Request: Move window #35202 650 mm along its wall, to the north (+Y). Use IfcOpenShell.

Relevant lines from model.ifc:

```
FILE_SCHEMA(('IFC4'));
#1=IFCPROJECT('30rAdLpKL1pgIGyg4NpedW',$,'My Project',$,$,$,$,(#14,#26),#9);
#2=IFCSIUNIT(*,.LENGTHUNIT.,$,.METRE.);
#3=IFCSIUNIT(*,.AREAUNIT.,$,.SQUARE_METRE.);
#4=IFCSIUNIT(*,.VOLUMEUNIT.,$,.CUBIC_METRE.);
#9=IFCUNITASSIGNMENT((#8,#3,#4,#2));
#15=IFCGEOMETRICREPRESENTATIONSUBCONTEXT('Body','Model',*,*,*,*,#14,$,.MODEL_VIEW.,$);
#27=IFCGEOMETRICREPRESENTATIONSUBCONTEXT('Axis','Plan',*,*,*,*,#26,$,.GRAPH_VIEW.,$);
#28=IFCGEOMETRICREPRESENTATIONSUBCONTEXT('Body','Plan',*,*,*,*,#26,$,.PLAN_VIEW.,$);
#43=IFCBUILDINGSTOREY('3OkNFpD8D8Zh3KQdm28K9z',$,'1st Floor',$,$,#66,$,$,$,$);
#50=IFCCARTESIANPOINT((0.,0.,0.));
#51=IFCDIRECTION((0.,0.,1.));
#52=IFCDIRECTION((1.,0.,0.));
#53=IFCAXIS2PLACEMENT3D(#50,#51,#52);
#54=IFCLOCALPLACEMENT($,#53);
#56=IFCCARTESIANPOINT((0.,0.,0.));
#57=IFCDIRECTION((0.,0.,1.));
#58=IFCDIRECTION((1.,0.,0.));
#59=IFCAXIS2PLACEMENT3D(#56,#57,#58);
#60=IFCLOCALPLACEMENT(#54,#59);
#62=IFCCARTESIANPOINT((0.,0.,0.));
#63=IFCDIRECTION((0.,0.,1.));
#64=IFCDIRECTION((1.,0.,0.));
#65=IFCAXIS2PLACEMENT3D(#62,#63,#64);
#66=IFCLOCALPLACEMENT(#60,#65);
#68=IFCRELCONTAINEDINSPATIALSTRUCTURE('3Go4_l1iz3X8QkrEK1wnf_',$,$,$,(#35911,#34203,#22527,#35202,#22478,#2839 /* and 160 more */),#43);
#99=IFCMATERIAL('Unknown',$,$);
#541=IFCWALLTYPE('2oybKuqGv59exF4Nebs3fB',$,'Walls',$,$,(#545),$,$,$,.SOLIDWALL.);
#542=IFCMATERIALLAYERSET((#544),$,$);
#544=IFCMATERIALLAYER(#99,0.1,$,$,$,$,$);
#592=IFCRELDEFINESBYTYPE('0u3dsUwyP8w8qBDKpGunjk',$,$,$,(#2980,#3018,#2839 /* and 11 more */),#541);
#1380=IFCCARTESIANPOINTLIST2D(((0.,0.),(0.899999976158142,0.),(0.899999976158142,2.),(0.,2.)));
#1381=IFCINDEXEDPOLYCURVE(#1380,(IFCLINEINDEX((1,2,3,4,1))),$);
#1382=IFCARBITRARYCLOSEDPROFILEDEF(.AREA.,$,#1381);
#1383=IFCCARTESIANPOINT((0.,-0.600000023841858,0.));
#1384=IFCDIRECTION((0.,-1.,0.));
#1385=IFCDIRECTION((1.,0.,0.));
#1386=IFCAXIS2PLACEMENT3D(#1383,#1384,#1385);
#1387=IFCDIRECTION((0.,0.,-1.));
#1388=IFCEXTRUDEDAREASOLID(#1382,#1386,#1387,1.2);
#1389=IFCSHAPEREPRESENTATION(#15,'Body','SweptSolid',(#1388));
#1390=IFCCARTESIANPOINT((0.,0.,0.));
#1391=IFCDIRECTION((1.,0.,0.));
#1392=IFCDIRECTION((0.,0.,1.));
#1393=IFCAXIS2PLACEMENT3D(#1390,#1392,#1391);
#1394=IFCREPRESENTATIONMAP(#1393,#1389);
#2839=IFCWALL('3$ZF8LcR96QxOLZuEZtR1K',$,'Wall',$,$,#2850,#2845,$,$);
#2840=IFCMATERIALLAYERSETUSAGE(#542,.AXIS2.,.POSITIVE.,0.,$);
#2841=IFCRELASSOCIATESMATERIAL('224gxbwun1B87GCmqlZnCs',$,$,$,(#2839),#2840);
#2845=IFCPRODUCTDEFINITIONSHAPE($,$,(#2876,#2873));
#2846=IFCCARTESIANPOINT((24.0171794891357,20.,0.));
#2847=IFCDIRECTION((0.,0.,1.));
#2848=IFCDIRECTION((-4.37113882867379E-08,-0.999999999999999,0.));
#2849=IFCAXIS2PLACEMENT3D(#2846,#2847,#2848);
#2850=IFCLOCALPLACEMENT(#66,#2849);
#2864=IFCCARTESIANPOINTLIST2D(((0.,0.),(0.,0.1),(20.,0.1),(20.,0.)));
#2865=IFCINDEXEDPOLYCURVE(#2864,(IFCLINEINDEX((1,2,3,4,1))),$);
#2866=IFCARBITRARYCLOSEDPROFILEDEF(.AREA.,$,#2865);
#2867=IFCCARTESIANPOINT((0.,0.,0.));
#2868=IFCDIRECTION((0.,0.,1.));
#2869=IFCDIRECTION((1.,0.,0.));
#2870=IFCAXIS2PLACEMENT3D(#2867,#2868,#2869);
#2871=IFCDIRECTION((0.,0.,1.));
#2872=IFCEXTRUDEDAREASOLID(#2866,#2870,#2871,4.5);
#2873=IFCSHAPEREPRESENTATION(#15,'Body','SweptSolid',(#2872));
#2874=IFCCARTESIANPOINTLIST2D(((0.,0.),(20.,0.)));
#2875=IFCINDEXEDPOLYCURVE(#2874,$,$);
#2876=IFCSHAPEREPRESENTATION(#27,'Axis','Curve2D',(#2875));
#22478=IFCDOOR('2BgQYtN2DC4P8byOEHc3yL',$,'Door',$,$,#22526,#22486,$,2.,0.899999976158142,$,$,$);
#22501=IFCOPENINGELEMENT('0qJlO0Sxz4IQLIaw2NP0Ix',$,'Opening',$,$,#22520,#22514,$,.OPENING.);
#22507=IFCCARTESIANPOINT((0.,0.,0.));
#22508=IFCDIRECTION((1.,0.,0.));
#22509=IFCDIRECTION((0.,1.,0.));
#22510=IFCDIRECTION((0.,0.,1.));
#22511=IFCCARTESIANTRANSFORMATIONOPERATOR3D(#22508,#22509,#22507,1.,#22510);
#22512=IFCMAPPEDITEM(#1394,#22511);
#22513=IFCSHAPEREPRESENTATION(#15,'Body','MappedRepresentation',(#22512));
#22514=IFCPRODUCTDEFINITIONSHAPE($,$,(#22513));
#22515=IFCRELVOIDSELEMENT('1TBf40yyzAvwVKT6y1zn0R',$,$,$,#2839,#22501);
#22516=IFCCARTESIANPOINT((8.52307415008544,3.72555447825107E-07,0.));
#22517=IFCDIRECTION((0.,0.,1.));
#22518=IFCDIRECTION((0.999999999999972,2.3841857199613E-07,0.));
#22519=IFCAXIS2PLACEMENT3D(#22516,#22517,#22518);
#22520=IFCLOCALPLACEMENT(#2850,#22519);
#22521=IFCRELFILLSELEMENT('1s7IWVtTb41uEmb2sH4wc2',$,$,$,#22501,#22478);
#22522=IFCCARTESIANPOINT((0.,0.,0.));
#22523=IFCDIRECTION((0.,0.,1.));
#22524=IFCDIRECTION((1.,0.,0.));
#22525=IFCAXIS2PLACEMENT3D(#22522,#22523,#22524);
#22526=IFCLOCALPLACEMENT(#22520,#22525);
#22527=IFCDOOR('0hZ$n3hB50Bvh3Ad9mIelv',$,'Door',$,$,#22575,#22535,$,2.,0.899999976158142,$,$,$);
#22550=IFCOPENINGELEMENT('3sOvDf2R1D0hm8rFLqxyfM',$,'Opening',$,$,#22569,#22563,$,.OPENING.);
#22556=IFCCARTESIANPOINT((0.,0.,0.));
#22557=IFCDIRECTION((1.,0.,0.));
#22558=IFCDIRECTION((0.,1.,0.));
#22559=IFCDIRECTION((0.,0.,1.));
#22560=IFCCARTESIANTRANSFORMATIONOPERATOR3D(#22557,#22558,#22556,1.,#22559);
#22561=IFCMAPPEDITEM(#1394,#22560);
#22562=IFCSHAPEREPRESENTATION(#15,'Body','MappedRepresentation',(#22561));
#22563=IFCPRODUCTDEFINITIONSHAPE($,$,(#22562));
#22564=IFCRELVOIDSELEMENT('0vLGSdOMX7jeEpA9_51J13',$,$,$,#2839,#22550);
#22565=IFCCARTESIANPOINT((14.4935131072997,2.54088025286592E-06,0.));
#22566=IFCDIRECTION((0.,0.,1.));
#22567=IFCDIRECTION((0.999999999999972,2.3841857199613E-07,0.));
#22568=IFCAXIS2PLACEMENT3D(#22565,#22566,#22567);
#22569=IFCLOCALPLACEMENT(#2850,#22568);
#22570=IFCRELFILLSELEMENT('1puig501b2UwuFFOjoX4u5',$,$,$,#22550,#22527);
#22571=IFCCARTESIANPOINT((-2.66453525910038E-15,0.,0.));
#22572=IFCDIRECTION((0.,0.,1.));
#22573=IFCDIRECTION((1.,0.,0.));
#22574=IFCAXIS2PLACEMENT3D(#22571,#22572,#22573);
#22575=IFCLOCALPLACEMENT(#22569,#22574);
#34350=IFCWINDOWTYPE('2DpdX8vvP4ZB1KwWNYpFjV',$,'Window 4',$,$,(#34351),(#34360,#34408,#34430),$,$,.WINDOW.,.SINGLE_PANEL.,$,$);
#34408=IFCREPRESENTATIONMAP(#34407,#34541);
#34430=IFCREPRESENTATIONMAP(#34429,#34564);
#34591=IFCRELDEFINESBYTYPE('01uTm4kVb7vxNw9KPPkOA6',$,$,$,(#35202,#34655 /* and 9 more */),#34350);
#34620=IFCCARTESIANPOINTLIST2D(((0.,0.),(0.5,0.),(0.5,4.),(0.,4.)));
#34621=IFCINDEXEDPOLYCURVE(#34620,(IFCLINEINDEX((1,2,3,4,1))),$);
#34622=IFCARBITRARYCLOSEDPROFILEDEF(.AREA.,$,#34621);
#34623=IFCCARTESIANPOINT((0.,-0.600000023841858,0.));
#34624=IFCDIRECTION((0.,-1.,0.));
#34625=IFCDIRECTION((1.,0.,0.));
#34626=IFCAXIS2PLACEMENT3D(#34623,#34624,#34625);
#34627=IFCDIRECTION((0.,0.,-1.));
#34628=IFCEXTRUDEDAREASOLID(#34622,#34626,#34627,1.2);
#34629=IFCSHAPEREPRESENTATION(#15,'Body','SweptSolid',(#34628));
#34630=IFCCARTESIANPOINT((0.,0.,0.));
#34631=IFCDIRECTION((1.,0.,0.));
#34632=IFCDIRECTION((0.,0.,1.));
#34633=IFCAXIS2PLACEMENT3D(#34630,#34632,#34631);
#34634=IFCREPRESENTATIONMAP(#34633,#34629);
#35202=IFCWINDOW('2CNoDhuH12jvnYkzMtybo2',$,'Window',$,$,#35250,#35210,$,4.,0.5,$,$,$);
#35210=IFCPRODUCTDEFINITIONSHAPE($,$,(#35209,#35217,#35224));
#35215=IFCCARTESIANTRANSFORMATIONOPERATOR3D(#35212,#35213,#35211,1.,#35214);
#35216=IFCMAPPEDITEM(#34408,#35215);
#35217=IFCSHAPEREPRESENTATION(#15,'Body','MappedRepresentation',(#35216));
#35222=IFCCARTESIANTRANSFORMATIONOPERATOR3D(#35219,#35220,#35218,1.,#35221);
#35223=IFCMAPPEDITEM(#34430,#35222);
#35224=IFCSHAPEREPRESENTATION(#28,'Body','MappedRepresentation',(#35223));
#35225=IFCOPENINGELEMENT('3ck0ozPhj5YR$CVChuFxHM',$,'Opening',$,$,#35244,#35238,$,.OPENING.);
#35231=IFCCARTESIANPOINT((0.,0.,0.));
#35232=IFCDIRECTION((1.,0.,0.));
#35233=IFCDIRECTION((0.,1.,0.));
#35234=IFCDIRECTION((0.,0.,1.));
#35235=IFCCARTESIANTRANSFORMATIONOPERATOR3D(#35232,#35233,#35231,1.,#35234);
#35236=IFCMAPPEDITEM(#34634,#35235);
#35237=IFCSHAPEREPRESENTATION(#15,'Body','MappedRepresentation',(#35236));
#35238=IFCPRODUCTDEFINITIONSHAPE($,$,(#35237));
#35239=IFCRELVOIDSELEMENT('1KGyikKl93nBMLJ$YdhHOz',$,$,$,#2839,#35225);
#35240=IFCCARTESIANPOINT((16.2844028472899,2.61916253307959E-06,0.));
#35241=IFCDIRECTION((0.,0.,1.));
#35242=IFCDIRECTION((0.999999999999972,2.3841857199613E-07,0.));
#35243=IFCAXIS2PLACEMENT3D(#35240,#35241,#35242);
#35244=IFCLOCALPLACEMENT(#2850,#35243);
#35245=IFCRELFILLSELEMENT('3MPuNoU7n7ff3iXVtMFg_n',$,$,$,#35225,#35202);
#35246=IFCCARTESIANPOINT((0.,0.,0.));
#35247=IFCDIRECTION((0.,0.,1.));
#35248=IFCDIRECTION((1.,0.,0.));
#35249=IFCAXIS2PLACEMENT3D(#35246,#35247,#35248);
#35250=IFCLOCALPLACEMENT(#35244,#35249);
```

```python
import ifcopenshell
import ifcopenshell.api.geometry
import ifcopenshell.util.placement

model = ifcopenshell.open("model.ifc")

window = model.by_guid("2CNoDhuH12jvnYkzMtybo2")
opening = window.FillsVoids[0].RelatingOpeningElement
wall = opening.VoidsElements[0].RelatingBuildingElement

wall_matrix = ifcopenshell.util.placement.get_local_placement(wall.ObjectPlacement)
shift = wall_matrix[:3, 0] * -0.65
before = ifcopenshell.util.placement.get_local_placement(window.ObjectPlacement)[:3, 3].copy()

# The window is placed relative to its opening, so it follows when the opening moves.
matrix = ifcopenshell.util.placement.get_local_placement(opening.ObjectPlacement)
matrix[:3, 3] += shift
ifcopenshell.api.geometry.edit_object_placement(
    model, product=opening, matrix=matrix, is_si=False, should_transform_children=True
)

after = ifcopenshell.util.placement.get_local_placement(window.ObjectPlacement)[:3, 3]
print("window moved by", (after - before).round(3) + 0.0)

model.write("model_v2.ifc")
```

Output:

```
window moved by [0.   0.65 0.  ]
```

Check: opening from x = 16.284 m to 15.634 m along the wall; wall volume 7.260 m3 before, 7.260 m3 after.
